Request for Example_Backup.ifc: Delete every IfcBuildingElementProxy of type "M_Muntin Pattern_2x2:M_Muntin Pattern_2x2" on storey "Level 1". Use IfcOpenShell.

First a look at what the model holds.

```python
import ifcopenshell
import ifcopenshell.util.element

model = ifcopenshell.open("Example_Backup.ifc")
print(model.schema)
storey = next(s for s in model.by_type("IfcBuildingStorey") if s.Name == "Level 1")
proxies = [e for e in ifcopenshell.util.element.get_decomposition(storey) if e.is_a("IfcBuildingElementProxy")]
seen = {}
for e in proxies:
    element_type = ifcopenshell.util.element.get_type(e)
    name = element_type.Name if element_type not in (None, e) else None
    seen[name] = seen.get(name, 0) + 1
for name, count in sorted(seen.items(), key=str):
    print(count, "x", name)
```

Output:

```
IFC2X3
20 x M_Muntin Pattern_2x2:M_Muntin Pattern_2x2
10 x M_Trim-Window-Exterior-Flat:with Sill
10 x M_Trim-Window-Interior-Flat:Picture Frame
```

```python
import ifcopenshell
import ifcopenshell.api.root
import ifcopenshell.util.element

model = ifcopenshell.open("Example_Backup.ifc")

storey = next(s for s in model.by_type("IfcBuildingStorey") if s.Name == "Level 1")
proxies = [e for e in ifcopenshell.util.element.get_decomposition(storey) if e.is_a("IfcBuildingElementProxy")]
targets = [e for e in proxies if (t := ifcopenshell.util.element.get_type(e)) not in (None, e) and t.Name == "M_Muntin Pattern_2x2:M_Muntin Pattern_2x2"]

for e in targets:
    ifcopenshell.api.root.remove_product(model, product=e)
print(len(targets), "removed")

model.write("Example_Backup-out.ifc")
```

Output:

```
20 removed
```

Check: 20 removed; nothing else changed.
